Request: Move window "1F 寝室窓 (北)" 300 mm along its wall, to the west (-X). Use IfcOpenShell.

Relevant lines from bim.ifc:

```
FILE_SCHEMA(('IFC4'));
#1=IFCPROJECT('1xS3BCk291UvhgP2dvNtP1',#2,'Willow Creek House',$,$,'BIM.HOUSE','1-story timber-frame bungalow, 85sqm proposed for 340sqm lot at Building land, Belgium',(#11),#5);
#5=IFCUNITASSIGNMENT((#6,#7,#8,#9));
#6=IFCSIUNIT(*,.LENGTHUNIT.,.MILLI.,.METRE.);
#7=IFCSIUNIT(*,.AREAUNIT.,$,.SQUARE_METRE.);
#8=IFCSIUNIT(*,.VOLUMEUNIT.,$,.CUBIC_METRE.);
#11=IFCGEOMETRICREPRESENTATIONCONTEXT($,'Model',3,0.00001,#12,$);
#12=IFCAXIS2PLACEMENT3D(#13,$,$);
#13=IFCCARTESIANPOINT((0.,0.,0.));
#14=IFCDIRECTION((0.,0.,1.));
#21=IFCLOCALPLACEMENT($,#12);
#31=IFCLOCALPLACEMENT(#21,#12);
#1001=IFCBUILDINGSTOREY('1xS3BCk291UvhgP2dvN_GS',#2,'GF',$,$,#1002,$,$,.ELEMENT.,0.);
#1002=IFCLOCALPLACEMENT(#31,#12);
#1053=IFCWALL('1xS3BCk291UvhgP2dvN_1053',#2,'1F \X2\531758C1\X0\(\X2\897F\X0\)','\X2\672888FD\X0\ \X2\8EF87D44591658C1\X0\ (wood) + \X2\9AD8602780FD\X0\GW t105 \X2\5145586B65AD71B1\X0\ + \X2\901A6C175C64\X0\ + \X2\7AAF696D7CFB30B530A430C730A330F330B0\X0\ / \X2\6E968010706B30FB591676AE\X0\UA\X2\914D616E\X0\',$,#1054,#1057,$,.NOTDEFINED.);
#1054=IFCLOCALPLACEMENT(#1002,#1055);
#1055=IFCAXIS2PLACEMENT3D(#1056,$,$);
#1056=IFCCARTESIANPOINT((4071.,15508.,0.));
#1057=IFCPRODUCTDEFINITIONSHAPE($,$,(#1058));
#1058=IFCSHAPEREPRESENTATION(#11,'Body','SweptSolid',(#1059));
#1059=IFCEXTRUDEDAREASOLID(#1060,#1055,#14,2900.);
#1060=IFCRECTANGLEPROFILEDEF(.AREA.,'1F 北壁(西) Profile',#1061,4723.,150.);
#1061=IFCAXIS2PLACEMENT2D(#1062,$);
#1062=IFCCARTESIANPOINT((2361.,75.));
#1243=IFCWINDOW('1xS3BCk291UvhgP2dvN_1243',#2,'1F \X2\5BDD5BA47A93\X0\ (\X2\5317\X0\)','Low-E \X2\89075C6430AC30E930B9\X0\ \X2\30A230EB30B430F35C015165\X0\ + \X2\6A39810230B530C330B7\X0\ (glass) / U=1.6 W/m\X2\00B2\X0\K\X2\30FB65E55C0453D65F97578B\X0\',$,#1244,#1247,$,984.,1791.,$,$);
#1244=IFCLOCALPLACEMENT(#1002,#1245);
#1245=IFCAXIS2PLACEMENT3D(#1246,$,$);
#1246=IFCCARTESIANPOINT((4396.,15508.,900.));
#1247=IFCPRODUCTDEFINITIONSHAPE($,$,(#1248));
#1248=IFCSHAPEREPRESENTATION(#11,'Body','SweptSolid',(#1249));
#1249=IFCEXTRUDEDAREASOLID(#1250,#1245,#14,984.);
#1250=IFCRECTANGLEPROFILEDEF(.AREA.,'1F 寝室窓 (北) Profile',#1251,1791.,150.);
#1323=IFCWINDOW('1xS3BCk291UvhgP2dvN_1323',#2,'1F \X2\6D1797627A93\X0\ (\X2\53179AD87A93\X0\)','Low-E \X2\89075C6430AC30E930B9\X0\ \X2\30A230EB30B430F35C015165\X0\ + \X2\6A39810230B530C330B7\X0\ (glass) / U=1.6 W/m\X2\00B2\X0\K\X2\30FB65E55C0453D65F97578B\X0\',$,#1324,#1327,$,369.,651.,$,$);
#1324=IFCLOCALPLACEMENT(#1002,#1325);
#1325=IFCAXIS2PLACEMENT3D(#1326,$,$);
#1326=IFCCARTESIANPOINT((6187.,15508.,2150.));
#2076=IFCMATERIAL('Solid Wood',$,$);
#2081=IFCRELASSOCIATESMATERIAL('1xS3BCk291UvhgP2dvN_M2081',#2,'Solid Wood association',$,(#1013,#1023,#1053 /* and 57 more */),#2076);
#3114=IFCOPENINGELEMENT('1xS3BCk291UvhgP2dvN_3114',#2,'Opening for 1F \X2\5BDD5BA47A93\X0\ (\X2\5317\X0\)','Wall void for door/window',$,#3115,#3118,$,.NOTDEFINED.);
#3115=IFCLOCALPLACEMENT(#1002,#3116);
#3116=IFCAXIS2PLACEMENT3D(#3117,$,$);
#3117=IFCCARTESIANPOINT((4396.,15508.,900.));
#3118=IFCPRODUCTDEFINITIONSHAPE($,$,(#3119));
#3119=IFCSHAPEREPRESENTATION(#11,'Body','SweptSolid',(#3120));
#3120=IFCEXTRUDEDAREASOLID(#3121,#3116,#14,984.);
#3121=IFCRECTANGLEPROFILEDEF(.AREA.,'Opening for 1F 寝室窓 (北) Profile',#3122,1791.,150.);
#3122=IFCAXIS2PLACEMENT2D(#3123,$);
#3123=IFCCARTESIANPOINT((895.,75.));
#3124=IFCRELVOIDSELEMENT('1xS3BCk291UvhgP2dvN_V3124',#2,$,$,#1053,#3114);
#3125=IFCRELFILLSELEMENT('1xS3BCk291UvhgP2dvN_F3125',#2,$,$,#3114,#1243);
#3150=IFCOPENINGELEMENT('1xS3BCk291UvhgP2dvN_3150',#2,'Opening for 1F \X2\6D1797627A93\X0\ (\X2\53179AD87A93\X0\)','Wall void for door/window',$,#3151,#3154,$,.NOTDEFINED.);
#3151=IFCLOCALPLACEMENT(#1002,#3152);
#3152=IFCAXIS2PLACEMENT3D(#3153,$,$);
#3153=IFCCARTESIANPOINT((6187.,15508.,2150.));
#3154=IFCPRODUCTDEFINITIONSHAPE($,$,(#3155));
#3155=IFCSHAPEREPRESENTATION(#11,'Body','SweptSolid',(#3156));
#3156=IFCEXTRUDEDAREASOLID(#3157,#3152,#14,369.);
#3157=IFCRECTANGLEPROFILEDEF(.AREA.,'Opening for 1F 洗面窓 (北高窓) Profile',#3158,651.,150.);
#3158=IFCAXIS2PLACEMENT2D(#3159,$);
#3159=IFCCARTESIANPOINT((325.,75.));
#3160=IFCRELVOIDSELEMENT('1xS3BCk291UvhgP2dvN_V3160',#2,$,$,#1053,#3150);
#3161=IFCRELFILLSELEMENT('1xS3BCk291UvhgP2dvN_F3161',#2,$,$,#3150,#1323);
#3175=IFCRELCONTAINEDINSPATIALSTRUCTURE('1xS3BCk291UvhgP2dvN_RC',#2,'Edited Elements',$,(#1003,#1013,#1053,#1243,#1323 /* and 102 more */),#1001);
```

```python
import ifcopenshell
import ifcopenshell.api.geometry
import ifcopenshell.util.placement
import ifcopenshell.util.unit

model = ifcopenshell.open("bim.ifc")
unit_scale = ifcopenshell.util.unit.calculate_unit_scale(model)

window = model.by_guid("1xS3BCk291UvhgP2dvN_1243")
opening = window.FillsVoids[0].RelatingOpeningElement
wall = opening.VoidsElements[0].RelatingBuildingElement

wall_matrix = ifcopenshell.util.placement.get_local_placement(wall.ObjectPlacement)
shift = wall_matrix[:3, 0] * -0.3 / unit_scale
before = ifcopenshell.util.placement.get_local_placement(window.ObjectPlacement)[:3, 3].copy()

# The window is not placed relative to its opening, so move both.
for product in (opening, window):
    matrix = ifcopenshell.util.placement.get_local_placement(product.ObjectPlacement)
    matrix[:3, 3] += shift
    ifcopenshell.api.geometry.edit_object_placement(model, product=product, matrix=matrix, is_si=False)

after = ifcopenshell.util.placement.get_local_placement(window.ObjectPlacement)[:3, 3]
print("window moved by", (after - before).round(3) + 0.0)

model.write("bim_rev.ifc")
```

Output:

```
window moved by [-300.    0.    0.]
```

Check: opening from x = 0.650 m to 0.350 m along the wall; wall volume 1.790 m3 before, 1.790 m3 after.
